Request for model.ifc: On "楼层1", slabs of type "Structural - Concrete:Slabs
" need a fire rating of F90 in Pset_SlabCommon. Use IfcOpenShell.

First a look at what the model holds.

```python
import ifcopenshell
import ifcopenshell.util.element

model = ifcopenshell.open("model.ifc")
print(model.schema)
storey = next(s for s in model.by_type("IfcBuildingStorey") if s.Name == "楼层1")
slabs = [e for e in ifcopenshell.util.element.get_decomposition(storey) if e.is_a("IfcSlab")]
seen = {}
for e in slabs:
    element_type = ifcopenshell.util.element.get_type(e)
    key = (element_type.Name if element_type != e and element_type else None, ifcopenshell.util.element.get_pset(e, "Pset_SlabCommon", "FireRating"))
    seen[key] = seen.get(key, 0) + 1
for (name, value), count in sorted(seen.items(), key=str):
    print(count, "x", name, "|", value)
```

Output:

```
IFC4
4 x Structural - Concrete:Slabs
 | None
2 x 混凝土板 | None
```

```python
import ifcopenshell
import ifcopenshell.api.pset
import ifcopenshell.util.element

model = ifcopenshell.open("model.ifc")

storey = next(s for s in model.by_type("IfcBuildingStorey") if s.Name == "楼层1")
slabs = [e for e in ifcopenshell.util.element.get_decomposition(storey) if e.is_a("IfcSlab")]

count = 0
for e in slabs:
    element_type = ifcopenshell.util.element.get_type(e)
    if element_type in (None, e) or element_type.Name != 'Structural - Concrete:Slabs\n':
        continue
    # add_pset returns the element's existing set when there is one.
    pset = ifcopenshell.api.pset.add_pset(model, product=e, name="Pset_SlabCommon")
    ifcopenshell.api.pset.edit_pset(model, pset=pset, properties={"FireRating": "F90"})
    count += 1

print(count, "slabs updated")

model.write("model_v2.ifc")
```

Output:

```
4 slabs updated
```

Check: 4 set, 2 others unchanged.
